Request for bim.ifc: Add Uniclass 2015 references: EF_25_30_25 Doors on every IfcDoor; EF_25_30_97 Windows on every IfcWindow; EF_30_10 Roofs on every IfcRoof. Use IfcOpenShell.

First a look at what the model holds.

```python
import ifcopenshell

model = ifcopenshell.open("bim.ifc")
print(model.schema)
print("classifications:", [c.Name for c in model.by_type("IfcClassification")])
for ifc_class in ("IfcDoor", "IfcRoof", "IfcStair", "IfcWall", "IfcWindow"):
    print(ifc_class, len(model.by_type(ifc_class)))
```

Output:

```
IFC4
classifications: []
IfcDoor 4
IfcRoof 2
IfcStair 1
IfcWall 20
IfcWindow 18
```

```python
import ifcopenshell
import ifcopenshell.api.classification

model = ifcopenshell.open("bim.ifc")

system = ifcopenshell.api.classification.add_classification(model, classification="Uniclass 2015")

codes = {
    "IfcDoor": ("EF_25_30_25", "Doors"),
    "IfcWindow": ("EF_25_30_97", "Windows"),
    "IfcRoof": ("EF_30_10", "Roofs"),
}
for ifc_class, (code, name) in codes.items():
    products = model.by_type(ifc_class)
    ifcopenshell.api.classification.add_reference(
        model, products=products, classification=system, identification=code, name=name
    )
    print(code, len(products))

model.write("bim_updated.ifc")
```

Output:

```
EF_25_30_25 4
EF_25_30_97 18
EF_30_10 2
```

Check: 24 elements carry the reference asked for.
